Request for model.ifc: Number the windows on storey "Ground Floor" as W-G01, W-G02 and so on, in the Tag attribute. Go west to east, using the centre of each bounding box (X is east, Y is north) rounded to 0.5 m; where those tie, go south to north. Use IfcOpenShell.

First a look at what the model holds.

```python
import ifcopenshell
import ifcopenshell.util.element
import ifcopenshell.util.placement

model = ifcopenshell.open("model.ifc")
print(model.schema)
storey = next(s for s in model.by_type("IfcBuildingStorey") if s.Name == "Ground Floor")
windows = [e for e in ifcopenshell.util.element.get_decomposition(storey) if e.is_a("IfcWindow")]
for e in sorted(windows, key=lambda e: e.id()):
    origin = ifcopenshell.util.placement.get_local_placement(e.ObjectPlacement)[:3, 3]
    print(e.id(), e.Tag, e.Name, origin.round(2) + 0.0, sep=" | ")
```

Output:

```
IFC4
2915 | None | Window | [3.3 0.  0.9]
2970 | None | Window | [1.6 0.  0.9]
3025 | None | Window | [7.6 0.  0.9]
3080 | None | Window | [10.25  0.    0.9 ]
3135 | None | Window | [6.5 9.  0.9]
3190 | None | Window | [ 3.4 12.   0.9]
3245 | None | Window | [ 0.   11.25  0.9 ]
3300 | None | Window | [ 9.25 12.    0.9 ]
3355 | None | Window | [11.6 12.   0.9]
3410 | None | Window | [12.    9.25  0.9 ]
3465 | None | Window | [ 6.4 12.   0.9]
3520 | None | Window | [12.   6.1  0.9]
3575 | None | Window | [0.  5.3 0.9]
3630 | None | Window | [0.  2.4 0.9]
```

```python
import ifcopenshell
import ifcopenshell.geom
import ifcopenshell.util.element
import ifcopenshell.util.shape

model = ifcopenshell.open("model.ifc")
settings = ifcopenshell.geom.settings()
settings.set("use-world-coords", True)


def centre(element):
    shape = ifcopenshell.geom.create_shape(settings, element)
    return ifcopenshell.util.shape.get_bbox_centroid(shape.geometry)


storey = next(s for s in model.by_type("IfcBuildingStorey") if s.Name == "Ground Floor")
windows = [e for e in ifcopenshell.util.element.get_decomposition(storey) if e.is_a("IfcWindow")]

# Insertion points can sit at a corner or the storey origin, so sort by the geometry (in metres).
centres = {e: centre(e) for e in windows}
windows.sort(key=lambda e: (round(centres[e][0] / 0.5), centres[e][1]))

for i, e in enumerate(windows, start=1):
    number = f"W-G{i:02d}"
    e.Tag = number
    print(e.id(), number)

model.write("model_rev.ifc")
```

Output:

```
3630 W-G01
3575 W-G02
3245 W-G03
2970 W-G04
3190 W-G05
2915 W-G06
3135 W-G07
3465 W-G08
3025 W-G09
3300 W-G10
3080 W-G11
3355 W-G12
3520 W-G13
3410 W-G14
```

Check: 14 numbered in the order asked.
